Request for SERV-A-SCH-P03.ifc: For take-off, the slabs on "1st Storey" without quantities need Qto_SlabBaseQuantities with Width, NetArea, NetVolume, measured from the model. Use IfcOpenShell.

First a look at what the model holds.

```python
import ifcopenshell
import ifcopenshell.util.element
import ifcopenshell.util.unit

model = ifcopenshell.open("SERV-A-SCH-P03.ifc")
print(model.schema)
for unit_type in ("LENGTHUNIT", "AREAUNIT", "VOLUMEUNIT"):
    print(unit_type, ifcopenshell.util.unit.calculate_unit_scale(model, unit_type))
storey = next(s for s in model.by_type("IfcBuildingStorey") if s.Name == "1st Storey")
slabs = [e for e in ifcopenshell.util.element.get_decomposition(storey) if e.is_a("IfcSlab")]
for e in sorted(slabs, key=lambda e: e.id()):
    print(e.id(), e.is_a(), e.Name, list(ifcopenshell.util.element.get_psets(e, qtos_only=True)), sep=" | ")
```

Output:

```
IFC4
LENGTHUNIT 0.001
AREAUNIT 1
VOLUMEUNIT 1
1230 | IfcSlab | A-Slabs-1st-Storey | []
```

```python
import ifcopenshell
import ifcopenshell.api.pset
import ifcopenshell.geom
import ifcopenshell.util.element
import ifcopenshell.util.shape
import ifcopenshell.util.unit

model = ifcopenshell.open("SERV-A-SCH-P03.ifc")
unit_scale = ifcopenshell.util.unit.calculate_unit_scale(model)
area_scale = ifcopenshell.util.unit.calculate_unit_scale(model, "AREAUNIT")
volume_scale = ifcopenshell.util.unit.calculate_unit_scale(model, "VOLUMEUNIT")
settings = ifcopenshell.geom.settings()

storey = next(s for s in model.by_type("IfcBuildingStorey") if s.Name == "1st Storey")
slabs = [e for e in ifcopenshell.util.element.get_decomposition(storey) if e.is_a("IfcSlab")]

for e in sorted(slabs, key=lambda e: e.id()):
    if ifcopenshell.util.element.get_psets(e, qtos_only=True, should_inherit=False):
        continue
    # Geometry comes back in metres, in the element's own axes.
    shape = ifcopenshell.geom.create_shape(settings, e)
    values = {
        "Width": ifcopenshell.util.shape.get_z(shape.geometry) / unit_scale,
        "NetArea": ifcopenshell.util.shape.get_footprint_area(shape.geometry) / area_scale,
        "NetVolume": ifcopenshell.util.shape.get_volume(shape.geometry) / volume_scale,
    }
    qto = ifcopenshell.api.pset.add_qto(model, product=e, name="Qto_SlabBaseQuantities")
    ifcopenshell.api.pset.edit_qto(model, qto=qto, properties=values)
    print(e.id(), {k: round(v, 3) for k, v in values.items()})

model.write("SERV-A-SCH-P03_rev.ifc")
```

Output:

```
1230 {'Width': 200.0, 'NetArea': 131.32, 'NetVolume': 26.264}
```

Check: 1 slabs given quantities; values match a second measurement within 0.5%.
